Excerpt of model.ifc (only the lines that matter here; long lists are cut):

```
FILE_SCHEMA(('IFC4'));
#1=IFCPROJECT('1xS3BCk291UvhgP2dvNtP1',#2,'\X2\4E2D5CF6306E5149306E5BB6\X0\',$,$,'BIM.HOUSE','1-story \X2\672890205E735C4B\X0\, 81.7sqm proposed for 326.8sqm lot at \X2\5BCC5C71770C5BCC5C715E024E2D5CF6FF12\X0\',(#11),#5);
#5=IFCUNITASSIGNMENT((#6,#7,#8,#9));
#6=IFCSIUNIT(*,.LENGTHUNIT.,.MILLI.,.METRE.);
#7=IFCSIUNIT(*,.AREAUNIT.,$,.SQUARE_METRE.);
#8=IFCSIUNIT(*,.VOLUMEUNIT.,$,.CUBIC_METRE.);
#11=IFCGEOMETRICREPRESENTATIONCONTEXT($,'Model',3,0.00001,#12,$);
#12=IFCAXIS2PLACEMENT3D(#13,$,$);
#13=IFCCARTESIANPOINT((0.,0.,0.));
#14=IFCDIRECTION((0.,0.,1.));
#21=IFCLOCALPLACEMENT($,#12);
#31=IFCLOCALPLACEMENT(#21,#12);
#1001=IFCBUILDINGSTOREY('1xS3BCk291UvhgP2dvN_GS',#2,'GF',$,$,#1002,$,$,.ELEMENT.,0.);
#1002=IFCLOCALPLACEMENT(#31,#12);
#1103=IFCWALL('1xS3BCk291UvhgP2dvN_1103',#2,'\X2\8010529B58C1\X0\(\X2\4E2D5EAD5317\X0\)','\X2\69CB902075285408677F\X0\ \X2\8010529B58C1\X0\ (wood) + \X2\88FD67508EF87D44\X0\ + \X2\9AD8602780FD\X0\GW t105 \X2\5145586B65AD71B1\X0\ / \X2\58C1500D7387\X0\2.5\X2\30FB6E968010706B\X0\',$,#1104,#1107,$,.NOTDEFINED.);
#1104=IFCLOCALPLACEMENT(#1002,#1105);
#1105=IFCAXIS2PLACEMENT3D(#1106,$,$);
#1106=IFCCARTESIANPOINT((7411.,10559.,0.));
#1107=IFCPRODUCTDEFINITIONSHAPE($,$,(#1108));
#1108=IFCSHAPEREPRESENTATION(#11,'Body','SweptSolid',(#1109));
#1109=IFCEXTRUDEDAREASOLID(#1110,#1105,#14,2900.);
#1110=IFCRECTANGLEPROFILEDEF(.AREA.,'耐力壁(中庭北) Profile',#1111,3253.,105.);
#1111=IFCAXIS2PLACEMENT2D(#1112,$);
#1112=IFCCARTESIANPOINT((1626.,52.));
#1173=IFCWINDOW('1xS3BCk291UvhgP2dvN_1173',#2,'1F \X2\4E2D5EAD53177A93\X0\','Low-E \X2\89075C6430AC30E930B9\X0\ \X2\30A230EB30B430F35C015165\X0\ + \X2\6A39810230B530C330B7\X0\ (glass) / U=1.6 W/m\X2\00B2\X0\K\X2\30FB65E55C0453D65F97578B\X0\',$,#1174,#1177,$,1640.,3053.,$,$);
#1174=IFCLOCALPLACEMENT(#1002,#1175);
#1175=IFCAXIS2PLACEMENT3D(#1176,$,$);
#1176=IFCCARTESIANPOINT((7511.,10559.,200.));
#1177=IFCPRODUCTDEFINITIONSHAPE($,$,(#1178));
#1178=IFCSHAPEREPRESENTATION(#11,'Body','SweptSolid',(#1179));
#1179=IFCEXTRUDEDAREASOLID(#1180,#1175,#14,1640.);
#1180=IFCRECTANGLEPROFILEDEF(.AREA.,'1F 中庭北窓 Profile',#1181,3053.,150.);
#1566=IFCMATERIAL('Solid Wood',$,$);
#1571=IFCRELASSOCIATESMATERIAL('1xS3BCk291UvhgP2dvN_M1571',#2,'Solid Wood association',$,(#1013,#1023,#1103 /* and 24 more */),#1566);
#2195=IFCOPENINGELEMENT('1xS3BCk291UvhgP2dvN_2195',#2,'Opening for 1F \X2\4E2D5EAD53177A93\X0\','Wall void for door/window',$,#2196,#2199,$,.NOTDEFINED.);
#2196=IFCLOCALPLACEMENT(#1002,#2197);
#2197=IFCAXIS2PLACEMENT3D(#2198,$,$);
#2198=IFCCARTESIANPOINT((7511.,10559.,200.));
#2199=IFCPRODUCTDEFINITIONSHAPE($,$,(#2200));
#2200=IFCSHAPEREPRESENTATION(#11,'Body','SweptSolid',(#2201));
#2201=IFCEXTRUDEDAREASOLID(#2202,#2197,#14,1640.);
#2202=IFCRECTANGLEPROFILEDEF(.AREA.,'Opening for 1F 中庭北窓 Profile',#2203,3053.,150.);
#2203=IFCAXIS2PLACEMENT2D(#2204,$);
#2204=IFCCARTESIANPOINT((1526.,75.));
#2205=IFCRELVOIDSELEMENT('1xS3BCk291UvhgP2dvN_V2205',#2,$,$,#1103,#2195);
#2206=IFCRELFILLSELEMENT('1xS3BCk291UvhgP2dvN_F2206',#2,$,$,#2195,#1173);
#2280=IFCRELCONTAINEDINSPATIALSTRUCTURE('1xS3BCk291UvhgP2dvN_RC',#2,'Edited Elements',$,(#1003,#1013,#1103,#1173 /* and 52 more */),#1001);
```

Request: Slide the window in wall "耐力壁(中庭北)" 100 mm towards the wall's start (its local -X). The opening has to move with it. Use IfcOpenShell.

```python
import ifcopenshell
import ifcopenshell.api.geometry
import ifcopenshell.util.placement

model = ifcopenshell.open("model.ifc")

window = model.by_id(1173)
opening = window.FillsVoids[0].RelatingOpeningElement
wall = opening.VoidsElements[0].RelatingBuildingElement

wall_matrix = ifcopenshell.util.placement.get_local_placement(wall.ObjectPlacement)
shift = wall_matrix[:3, 0] * -100.0
before = ifcopenshell.util.placement.get_local_placement(window.ObjectPlacement)[:3, 3].copy()

# The window is not placed relative to its opening, so move both.
for product in (opening, window):
    matrix = ifcopenshell.util.placement.get_local_placement(product.ObjectPlacement)
    matrix[:3, 3] += shift
    ifcopenshell.api.geometry.edit_object_placement(model, product=product, matrix=matrix, is_si=False)

after = ifcopenshell.util.placement.get_local_placement(window.ObjectPlacement)[:3, 3]
print("window moved by", (after - before).round(3) + 0.0)

model.write("model_edited.ifc")
```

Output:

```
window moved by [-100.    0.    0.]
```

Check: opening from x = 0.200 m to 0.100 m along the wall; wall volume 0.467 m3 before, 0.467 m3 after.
